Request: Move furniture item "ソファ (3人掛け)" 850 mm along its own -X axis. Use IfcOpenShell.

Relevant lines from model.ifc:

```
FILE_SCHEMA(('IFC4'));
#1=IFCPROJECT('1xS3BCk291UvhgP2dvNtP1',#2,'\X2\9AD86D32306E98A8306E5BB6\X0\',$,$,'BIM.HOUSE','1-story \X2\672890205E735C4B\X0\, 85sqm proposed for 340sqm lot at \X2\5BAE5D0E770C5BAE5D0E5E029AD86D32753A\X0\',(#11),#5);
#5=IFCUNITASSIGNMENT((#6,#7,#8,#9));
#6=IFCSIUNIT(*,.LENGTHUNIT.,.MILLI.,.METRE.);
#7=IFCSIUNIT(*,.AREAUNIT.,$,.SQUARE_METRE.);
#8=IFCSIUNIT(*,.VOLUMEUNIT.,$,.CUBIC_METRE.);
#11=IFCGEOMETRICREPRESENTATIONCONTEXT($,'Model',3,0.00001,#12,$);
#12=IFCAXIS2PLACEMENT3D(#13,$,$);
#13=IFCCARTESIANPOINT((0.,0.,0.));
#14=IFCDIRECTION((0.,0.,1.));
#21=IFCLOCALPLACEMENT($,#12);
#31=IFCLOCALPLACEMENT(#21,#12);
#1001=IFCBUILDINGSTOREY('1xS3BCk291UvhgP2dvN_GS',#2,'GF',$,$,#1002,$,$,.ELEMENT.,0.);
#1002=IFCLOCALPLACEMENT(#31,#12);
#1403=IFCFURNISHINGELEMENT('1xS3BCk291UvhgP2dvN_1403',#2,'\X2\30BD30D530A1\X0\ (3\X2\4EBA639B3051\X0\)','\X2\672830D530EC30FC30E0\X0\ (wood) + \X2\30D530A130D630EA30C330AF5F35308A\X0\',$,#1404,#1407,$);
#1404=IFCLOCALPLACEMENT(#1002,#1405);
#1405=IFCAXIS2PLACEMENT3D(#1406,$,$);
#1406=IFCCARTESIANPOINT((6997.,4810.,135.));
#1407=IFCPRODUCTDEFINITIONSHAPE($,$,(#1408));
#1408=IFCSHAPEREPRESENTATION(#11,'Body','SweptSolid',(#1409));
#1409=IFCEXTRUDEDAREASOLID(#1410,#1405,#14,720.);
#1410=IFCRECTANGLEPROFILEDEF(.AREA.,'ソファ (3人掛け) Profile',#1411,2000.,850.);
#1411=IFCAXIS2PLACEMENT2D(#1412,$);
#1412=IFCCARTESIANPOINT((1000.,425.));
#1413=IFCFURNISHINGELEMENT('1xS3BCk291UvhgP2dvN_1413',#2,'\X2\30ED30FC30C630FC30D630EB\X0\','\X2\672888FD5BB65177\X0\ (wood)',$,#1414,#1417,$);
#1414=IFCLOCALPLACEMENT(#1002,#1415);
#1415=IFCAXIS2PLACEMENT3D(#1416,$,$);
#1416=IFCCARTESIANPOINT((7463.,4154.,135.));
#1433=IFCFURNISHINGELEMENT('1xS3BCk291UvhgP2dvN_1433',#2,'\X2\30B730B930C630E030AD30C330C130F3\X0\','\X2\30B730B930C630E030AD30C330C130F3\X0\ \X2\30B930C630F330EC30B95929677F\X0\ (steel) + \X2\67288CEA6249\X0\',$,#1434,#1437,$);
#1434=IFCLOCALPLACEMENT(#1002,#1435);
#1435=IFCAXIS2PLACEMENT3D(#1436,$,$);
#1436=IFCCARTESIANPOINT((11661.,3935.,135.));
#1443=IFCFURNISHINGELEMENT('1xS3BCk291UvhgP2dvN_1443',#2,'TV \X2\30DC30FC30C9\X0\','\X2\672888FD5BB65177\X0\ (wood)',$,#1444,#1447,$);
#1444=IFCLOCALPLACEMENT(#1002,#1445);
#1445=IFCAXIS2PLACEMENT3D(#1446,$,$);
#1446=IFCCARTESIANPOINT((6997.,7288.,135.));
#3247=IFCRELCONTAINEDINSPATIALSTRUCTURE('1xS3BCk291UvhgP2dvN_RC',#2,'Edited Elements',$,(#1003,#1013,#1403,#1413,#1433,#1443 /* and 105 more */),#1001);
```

```python
import ifcopenshell
import ifcopenshell.api.geometry
import ifcopenshell.util.placement
import ifcopenshell.util.unit

model = ifcopenshell.open("model.ifc")
unit_scale = ifcopenshell.util.unit.calculate_unit_scale(model)

item = model.by_guid("1xS3BCk291UvhgP2dvN_1403")
matrix = ifcopenshell.util.placement.get_local_placement(item.ObjectPlacement)
matrix[:3, 3] -= matrix[:3, 0] * 0.85 / unit_scale
ifcopenshell.api.geometry.edit_object_placement(model, product=item, matrix=matrix, is_si=False)

print(ifcopenshell.util.placement.get_local_placement(item.ObjectPlacement).round(3) + 0.0)

model.write("model-out.ifc")
```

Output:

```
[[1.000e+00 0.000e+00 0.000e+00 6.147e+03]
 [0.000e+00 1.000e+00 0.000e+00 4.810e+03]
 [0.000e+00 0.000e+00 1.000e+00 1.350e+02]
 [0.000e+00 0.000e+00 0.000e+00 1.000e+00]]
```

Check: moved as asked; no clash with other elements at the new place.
